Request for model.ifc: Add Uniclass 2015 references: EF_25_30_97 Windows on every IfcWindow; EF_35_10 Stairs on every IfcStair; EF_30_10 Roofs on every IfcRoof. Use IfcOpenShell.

First a look at what the model holds.

```python
import ifcopenshell

model = ifcopenshell.open("model.ifc")
print(model.schema)
print("classifications:", [c.Name for c in model.by_type("IfcClassification")])
for ifc_class in ("IfcDoor", "IfcRoof", "IfcStair", "IfcWall", "IfcWindow"):
    print(ifc_class, len(model.by_type(ifc_class)))
```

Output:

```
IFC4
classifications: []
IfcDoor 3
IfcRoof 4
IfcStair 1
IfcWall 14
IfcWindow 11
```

```python
import ifcopenshell
import ifcopenshell.api.classification

model = ifcopenshell.open("model.ifc")

system = ifcopenshell.api.classification.add_classification(model, classification="Uniclass 2015")

codes = {
    "IfcWindow": ("EF_25_30_97", "Windows"),
    "IfcStair": ("EF_35_10", "Stairs"),
    "IfcRoof": ("EF_30_10", "Roofs"),
}
for ifc_class, (code, name) in codes.items():
    products = model.by_type(ifc_class)
    ifcopenshell.api.classification.add_reference(
        model, products=products, classification=system, identification=code, name=name
    )
    print(code, len(products))

model.write("model_edited.ifc")
```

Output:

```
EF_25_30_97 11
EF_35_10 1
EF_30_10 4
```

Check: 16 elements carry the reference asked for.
